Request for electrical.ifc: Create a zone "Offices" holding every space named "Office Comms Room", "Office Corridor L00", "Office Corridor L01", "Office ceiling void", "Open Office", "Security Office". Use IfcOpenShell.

First a look at what the model holds.

```python
import ifcopenshell

model = ifcopenshell.open("electrical.ifc")
print(model.schema)
seen = {}
for space in model.by_type("IfcSpace"):
    seen[space.LongName] = seen.get(space.LongName, 0) + 1
for name, count in sorted(seen.items(), key=str):
    print(count, "x", name)
print("zones:", [z.Name for z in model.by_type("IfcZone")][:20])
```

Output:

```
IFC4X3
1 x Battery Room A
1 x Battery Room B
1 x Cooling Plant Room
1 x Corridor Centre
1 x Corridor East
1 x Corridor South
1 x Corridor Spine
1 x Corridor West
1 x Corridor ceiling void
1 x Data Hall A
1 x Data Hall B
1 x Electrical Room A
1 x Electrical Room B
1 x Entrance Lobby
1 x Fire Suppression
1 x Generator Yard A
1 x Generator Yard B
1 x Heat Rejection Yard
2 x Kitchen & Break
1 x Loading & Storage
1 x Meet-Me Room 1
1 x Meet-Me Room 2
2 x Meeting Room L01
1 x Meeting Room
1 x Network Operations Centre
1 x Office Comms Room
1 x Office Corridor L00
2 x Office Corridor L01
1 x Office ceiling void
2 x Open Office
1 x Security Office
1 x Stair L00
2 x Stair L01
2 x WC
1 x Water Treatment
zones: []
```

```python
import ifcopenshell
import ifcopenshell.api.group
import ifcopenshell.api.root

model = ifcopenshell.open("electrical.ifc")

names = {"Office Comms Room", "Office Corridor L00", "Office Corridor L01", "Office ceiling void", "Open Office", "Security Office"}
spaces = [s for s in model.by_type("IfcSpace") if s.LongName in names]

zone = ifcopenshell.api.root.create_entity(model, ifc_class="IfcZone", name="Offices")
ifcopenshell.api.group.assign_group(model, products=spaces, group=zone)
print(len(spaces), "spaces in", zone.Name)

model.write("electrical_updated.ifc")
```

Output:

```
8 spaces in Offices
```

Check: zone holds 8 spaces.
